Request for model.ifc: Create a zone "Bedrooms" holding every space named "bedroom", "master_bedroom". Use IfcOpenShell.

First a look at what the model holds.

```python
import ifcopenshell

model = ifcopenshell.open("model.ifc")
print(model.schema)
seen = {}
for space in model.by_type("IfcSpace"):
    seen[space.LongName] = seen.get(space.LongName, 0) + 1
for name, count in sorted(seen.items(), key=str):
    print(count, "x", name)
print("zones:", [z.Name for z in model.by_type("IfcZone")][:20])
```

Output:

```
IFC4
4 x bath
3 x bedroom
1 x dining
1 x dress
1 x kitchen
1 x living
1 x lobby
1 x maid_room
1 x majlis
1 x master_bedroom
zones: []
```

```python
import ifcopenshell
import ifcopenshell.api.group
import ifcopenshell.api.root

model = ifcopenshell.open("model.ifc")

names = {"bedroom", "master_bedroom"}
spaces = [s for s in model.by_type("IfcSpace") if s.LongName in names]

zone = ifcopenshell.api.root.create_entity(model, ifc_class="IfcZone", name="Bedrooms")
ifcopenshell.api.group.assign_group(model, products=spaces, group=zone)
print(len(spaces), "spaces in", zone.Name)

model.write("model_rev.ifc")
```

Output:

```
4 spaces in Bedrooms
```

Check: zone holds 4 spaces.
